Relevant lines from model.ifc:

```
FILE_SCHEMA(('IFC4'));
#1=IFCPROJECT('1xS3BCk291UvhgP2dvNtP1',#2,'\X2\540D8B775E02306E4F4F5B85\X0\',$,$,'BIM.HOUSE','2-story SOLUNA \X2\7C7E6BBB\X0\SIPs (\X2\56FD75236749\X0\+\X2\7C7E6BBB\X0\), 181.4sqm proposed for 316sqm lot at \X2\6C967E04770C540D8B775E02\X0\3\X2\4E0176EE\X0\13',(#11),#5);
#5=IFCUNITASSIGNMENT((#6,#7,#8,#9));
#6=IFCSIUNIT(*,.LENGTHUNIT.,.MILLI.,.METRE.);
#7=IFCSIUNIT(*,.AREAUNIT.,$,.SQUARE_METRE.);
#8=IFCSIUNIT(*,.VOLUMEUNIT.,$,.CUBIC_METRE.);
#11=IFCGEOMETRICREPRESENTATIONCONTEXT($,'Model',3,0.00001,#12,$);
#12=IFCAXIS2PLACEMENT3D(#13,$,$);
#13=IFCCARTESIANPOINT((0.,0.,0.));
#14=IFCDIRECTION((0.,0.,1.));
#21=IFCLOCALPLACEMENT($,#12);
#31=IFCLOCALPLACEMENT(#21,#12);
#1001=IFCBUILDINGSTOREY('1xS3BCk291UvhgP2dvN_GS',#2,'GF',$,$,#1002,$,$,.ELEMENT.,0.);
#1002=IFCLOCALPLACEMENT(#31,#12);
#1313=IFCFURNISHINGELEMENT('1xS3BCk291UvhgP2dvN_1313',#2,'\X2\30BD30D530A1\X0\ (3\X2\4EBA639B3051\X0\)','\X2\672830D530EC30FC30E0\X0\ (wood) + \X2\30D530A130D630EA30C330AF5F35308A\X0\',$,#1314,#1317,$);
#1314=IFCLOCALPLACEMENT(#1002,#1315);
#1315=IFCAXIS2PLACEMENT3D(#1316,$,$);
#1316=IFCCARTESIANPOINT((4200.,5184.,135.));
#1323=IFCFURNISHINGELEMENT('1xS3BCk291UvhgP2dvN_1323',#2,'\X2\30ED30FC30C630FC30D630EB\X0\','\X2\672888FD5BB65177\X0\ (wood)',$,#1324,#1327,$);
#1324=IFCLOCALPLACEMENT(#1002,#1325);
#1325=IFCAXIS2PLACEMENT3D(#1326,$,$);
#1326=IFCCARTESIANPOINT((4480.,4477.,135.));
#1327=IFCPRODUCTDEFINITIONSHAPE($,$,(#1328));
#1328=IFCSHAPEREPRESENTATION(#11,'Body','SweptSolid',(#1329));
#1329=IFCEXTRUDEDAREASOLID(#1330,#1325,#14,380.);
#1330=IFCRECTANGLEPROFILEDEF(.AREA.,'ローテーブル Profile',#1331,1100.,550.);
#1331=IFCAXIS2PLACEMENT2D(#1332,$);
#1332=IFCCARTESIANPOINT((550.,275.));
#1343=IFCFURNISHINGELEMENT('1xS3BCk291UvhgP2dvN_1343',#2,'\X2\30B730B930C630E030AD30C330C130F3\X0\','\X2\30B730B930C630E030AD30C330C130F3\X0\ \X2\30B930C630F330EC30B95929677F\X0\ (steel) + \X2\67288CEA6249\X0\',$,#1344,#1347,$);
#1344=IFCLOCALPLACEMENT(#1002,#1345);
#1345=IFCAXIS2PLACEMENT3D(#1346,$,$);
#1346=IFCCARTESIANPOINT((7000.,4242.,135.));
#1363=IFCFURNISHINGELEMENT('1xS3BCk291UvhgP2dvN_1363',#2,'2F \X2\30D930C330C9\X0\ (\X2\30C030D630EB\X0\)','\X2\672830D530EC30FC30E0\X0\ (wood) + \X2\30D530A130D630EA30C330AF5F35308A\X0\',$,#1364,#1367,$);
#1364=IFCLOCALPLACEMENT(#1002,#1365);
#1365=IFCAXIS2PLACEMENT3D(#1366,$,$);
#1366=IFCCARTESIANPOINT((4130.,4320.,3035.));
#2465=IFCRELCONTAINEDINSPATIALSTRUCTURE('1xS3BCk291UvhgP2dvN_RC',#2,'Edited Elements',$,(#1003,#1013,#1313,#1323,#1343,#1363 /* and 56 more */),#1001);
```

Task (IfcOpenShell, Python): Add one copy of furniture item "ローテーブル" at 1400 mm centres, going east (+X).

```python
import numpy as np
import ifcopenshell
import ifcopenshell.api.geometry
import ifcopenshell.api.root
import ifcopenshell.util.element
import ifcopenshell.util.placement

model = ifcopenshell.open("model.ifc")


def reuse_history(source, copy):
    """copy_class also copies each property set's owner history, people and application; keep the originals."""
    for rel in copy.IsDefinedBy:
        if rel.is_a("IfcRelDefinesByProperties") and (history := rel.RelatingPropertyDefinition.OwnerHistory):
            rel.RelatingPropertyDefinition.OwnerHistory = source.OwnerHistory
            ifcopenshell.util.element.remove_deep2(model, history)


source = model.by_guid("1xS3BCk291UvhgP2dvN_1323")
base = ifcopenshell.util.placement.get_local_placement(source.ObjectPlacement)
step = np.array([1.0, 0.0, 0.0]) * 1400.0

for i in range(1, 2):
    copy = ifcopenshell.api.root.copy_class(model, product=source)
    copy.Representation = ifcopenshell.util.element.copy_deep(
        model, source.Representation, exclude=["IfcGeometricRepresentationContext", "IfcRepresentationMap"]
    )
    reuse_history(source, copy)
    matrix = base.copy()
    matrix[:3, 3] += i * step
    print("added at", matrix[:3, 3].round(3) + 0.0)
    ifcopenshell.api.geometry.edit_object_placement(model, product=copy, matrix=matrix, is_si=False)

model.write("model_edited.ifc")
```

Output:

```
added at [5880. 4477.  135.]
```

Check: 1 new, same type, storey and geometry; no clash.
